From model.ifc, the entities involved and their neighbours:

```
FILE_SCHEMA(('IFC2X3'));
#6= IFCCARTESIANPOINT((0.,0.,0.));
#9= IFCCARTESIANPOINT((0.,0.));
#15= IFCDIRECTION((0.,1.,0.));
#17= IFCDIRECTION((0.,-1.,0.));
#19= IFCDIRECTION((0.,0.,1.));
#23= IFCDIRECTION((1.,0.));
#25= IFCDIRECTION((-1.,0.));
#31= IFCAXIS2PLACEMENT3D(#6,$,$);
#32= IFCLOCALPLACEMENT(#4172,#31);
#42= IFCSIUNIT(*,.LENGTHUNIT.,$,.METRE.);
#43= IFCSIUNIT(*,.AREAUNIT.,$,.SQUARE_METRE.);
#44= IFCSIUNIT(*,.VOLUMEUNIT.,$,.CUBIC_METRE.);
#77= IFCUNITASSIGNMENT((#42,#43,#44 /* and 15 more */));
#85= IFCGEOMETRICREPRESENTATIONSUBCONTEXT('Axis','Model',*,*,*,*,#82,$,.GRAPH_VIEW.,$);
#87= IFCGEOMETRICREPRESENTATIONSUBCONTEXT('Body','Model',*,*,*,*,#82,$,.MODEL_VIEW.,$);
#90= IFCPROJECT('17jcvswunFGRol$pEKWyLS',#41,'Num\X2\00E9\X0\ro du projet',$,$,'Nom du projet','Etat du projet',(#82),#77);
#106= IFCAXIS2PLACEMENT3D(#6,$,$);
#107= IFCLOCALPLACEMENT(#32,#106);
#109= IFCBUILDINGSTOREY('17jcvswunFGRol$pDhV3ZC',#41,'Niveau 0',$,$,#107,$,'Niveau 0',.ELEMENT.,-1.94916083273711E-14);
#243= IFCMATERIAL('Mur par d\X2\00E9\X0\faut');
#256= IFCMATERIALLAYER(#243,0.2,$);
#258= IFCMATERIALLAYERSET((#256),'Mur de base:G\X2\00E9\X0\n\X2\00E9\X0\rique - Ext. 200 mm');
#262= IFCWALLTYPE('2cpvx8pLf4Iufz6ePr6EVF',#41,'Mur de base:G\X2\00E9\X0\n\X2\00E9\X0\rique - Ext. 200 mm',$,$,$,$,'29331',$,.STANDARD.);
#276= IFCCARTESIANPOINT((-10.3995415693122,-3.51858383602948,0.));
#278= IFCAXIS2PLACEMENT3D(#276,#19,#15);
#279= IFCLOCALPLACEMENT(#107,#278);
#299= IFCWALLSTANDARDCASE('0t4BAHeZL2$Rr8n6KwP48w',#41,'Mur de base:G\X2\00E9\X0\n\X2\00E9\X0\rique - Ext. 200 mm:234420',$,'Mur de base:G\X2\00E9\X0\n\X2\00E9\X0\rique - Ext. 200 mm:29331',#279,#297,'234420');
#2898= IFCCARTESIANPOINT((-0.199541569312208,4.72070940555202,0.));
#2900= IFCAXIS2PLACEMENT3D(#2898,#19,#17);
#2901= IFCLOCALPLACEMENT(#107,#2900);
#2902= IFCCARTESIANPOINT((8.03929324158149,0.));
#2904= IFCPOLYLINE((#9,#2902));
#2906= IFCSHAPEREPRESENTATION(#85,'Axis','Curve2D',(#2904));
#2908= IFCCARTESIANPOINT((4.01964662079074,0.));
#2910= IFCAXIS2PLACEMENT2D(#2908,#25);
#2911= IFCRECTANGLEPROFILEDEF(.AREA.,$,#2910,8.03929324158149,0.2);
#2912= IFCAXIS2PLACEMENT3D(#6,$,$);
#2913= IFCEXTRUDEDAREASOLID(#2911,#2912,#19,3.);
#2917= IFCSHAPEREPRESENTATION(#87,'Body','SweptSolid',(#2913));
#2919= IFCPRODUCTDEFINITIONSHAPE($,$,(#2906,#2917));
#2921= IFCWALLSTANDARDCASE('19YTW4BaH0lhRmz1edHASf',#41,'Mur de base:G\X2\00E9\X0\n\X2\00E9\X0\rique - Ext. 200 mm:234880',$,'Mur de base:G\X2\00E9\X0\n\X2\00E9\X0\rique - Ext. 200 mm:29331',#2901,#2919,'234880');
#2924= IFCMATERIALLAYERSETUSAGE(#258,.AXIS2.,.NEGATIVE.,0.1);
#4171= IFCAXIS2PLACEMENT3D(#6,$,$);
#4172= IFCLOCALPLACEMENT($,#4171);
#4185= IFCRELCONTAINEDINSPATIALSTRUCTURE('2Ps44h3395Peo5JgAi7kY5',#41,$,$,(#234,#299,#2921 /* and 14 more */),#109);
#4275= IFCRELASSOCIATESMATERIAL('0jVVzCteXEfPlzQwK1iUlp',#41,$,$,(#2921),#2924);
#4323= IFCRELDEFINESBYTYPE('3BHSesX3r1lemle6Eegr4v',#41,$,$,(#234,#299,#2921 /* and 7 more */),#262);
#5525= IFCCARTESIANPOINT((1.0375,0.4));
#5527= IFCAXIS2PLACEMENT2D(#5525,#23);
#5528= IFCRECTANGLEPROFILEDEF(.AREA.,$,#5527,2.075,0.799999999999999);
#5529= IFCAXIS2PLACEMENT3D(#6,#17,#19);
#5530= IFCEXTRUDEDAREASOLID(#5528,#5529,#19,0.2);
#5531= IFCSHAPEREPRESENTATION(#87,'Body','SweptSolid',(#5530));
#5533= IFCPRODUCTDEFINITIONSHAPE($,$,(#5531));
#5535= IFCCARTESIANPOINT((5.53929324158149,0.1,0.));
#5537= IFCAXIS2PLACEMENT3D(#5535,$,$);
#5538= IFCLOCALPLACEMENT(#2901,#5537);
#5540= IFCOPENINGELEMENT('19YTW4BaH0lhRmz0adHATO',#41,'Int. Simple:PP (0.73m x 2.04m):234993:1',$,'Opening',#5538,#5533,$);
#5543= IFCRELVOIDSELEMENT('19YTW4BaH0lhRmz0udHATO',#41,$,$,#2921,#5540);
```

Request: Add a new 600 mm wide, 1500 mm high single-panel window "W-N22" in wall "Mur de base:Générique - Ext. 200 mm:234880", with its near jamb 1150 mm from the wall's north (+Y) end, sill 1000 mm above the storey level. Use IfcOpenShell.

```python
import numpy as np
import ifcopenshell
import ifcopenshell.api.feature
import ifcopenshell.api.geometry
import ifcopenshell.api.root
import ifcopenshell.api.spatial
import ifcopenshell.api.type
import ifcopenshell.geom
import ifcopenshell.util.element
import ifcopenshell.util.placement
import ifcopenshell.util.representation
import ifcopenshell.util.shape
import ifcopenshell.util.unit

model = ifcopenshell.open("model.ifc")
unit_scale = ifcopenshell.util.unit.calculate_unit_scale(model)
settings = ifcopenshell.geom.settings()


def volume(element):
    """Net volume in cubic metres, openings subtracted."""
    shape = ifcopenshell.geom.create_shape(settings, element)
    return ifcopenshell.util.shape.get_volume(shape.geometry)


wall = model.by_guid("19YTW4BaH0lhRmz1edHASf")
storey = ifcopenshell.util.element.get_container(wall, ifc_class="IfcBuildingStorey")
context = ifcopenshell.util.representation.get_context(model, "Model", "Body", "MODEL_VIEW")
before = volume(wall)

width, height, from_end, sill = 0.6, 1.5, 1.15, 1  # metres

# The wall runs along its own X axis, and the end named is its -X end.
wall_shape = ifcopenshell.geom.create_shape(settings, wall)
x, y, z = ifcopenshell.util.shape.get_vertices(wall_shape.geometry).T
start = x.min() + from_end
face, thickness = float(y.min()), float(y.max() - y.min())
wall_matrix = ifcopenshell.util.placement.get_local_placement(wall.ObjectPlacement)
level = ifcopenshell.util.placement.get_local_placement(storey.ObjectPlacement)[2, 3]


def in_wall(x, y):
    """Placement at x, y metres in the wall's axes, at sill height."""
    matrix = wall_matrix.copy()
    matrix[:, 3] = wall_matrix @ np.array([x / unit_scale, y / unit_scale, 0.0, 1.0])
    matrix[2, 3] = level + sill / unit_scale
    return matrix


# Opening: a box that overshoots both wall faces by 50 mm.
opening = ifcopenshell.api.root.create_entity(model, ifc_class="IfcOpeningElement")
box = ifcopenshell.api.geometry.add_wall_representation(
    model, context=context, length=width, height=height, thickness=thickness + 0.1
)
ifcopenshell.api.geometry.assign_representation(model, product=opening, representation=box)
ifcopenshell.api.geometry.edit_object_placement(model, product=opening, matrix=in_wall(start, face - 0.05), is_si=False)
ifcopenshell.api.feature.add_feature(model, feature=opening, element=wall)

window = ifcopenshell.api.root.create_entity(model, ifc_class="IfcWindow", name="W-N22")
window.OverallWidth, window.OverallHeight = width / unit_scale, height / unit_scale
body = ifcopenshell.api.geometry.add_window_representation(
    model,
    context=context,
    overall_width=window.OverallWidth,
    overall_height=window.OverallHeight,
    partition_type="SINGLE_PANEL",
)
ifcopenshell.api.geometry.assign_representation(model, product=window, representation=body)
ifcopenshell.api.spatial.assign_container(model, products=[window], relating_structure=storey)
fills = ifcopenshell.api.feature.add_filling(model, opening=opening, element=window)
fills.OwnerHistory = window.OwnerHistory  # required in IFC2X3

# IFC2X3 keeps the operation on the window style.
style = ifcopenshell.api.root.create_entity(model, ifc_class="IfcWindowStyle", name="W-N22")
style.OperationType, style.ConstructionType = "SINGLE_PANEL", "NOTDEFINED"
style.ParameterTakesPrecedence = style.Sizeable = False
ifcopenshell.api.type.assign_type(model, related_objects=[window], relating_type=style)

# Centre the window in the wall's thickness.
ifcopenshell.api.geometry.edit_object_placement(model, product=window, matrix=in_wall(start, face), is_si=False)
window_shape = ifcopenshell.geom.create_shape(settings, window)
depth = ifcopenshell.util.shape.get_vertices(window_shape.geometry)[:, 1]
offset = face + thickness / 2 - (depth.min() + depth.max()) / 2
ifcopenshell.api.geometry.edit_object_placement(model, product=window, matrix=in_wall(start, offset), is_si=False)

after = volume(wall)

print(f"wall volume {before:.3f} -> {after:.3f} m3")

model.write("model_rev.ifc")
```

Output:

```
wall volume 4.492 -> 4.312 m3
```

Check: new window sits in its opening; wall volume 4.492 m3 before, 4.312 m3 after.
